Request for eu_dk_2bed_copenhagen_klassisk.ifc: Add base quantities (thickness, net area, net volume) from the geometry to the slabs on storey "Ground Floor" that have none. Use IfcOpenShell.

First a look at what the model holds.

```python
import ifcopenshell
import ifcopenshell.util.element
import ifcopenshell.util.unit

model = ifcopenshell.open("eu_dk_2bed_copenhagen_klassisk.ifc")
print(model.schema)
for unit_type in ("LENGTHUNIT", "AREAUNIT", "VOLUMEUNIT"):
    print(unit_type, ifcopenshell.util.unit.calculate_unit_scale(model, unit_type))
storey = next(s for s in model.by_type("IfcBuildingStorey") if s.Name == "Ground Floor")
slabs = [e for e in ifcopenshell.util.element.get_decomposition(storey) if e.is_a("IfcSlab")]
for e in sorted(slabs, key=lambda e: e.id()):
    print(e.id(), e.is_a(), e.Name, list(ifcopenshell.util.element.get_psets(e, qtos_only=True)), sep=" | ")
```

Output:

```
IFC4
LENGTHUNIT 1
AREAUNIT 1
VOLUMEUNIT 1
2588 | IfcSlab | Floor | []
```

```python
import ifcopenshell
import ifcopenshell.api.pset
import ifcopenshell.geom
import ifcopenshell.util.element
import ifcopenshell.util.shape
import ifcopenshell.util.unit

model = ifcopenshell.open("eu_dk_2bed_copenhagen_klassisk.ifc")
unit_scale = ifcopenshell.util.unit.calculate_unit_scale(model)
area_scale = ifcopenshell.util.unit.calculate_unit_scale(model, "AREAUNIT")
volume_scale = ifcopenshell.util.unit.calculate_unit_scale(model, "VOLUMEUNIT")
settings = ifcopenshell.geom.settings()

storey = next(s for s in model.by_type("IfcBuildingStorey") if s.Name == "Ground Floor")
slabs = [e for e in ifcopenshell.util.element.get_decomposition(storey) if e.is_a("IfcSlab")]

for e in sorted(slabs, key=lambda e: e.id()):
    if ifcopenshell.util.element.get_psets(e, qtos_only=True, should_inherit=False):
        continue
    # Geometry comes back in metres, in the element's own axes.
    shape = ifcopenshell.geom.create_shape(settings, e)
    values = {
        "Width": ifcopenshell.util.shape.get_z(shape.geometry) / unit_scale,
        "NetArea": ifcopenshell.util.shape.get_footprint_area(shape.geometry) / area_scale,
        "NetVolume": ifcopenshell.util.shape.get_volume(shape.geometry) / volume_scale,
    }
    qto = ifcopenshell.api.pset.add_qto(model, product=e, name="Qto_SlabBaseQuantities")
    ifcopenshell.api.pset.edit_qto(model, qto=qto, properties=values)
    print(e.id(), {k: round(v, 3) for k, v in values.items()})

model.write("eu_dk_2bed_copenhagen_klassisk_rev.ifc")
```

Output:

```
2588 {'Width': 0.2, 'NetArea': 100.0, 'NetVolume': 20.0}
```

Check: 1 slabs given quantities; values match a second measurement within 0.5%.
